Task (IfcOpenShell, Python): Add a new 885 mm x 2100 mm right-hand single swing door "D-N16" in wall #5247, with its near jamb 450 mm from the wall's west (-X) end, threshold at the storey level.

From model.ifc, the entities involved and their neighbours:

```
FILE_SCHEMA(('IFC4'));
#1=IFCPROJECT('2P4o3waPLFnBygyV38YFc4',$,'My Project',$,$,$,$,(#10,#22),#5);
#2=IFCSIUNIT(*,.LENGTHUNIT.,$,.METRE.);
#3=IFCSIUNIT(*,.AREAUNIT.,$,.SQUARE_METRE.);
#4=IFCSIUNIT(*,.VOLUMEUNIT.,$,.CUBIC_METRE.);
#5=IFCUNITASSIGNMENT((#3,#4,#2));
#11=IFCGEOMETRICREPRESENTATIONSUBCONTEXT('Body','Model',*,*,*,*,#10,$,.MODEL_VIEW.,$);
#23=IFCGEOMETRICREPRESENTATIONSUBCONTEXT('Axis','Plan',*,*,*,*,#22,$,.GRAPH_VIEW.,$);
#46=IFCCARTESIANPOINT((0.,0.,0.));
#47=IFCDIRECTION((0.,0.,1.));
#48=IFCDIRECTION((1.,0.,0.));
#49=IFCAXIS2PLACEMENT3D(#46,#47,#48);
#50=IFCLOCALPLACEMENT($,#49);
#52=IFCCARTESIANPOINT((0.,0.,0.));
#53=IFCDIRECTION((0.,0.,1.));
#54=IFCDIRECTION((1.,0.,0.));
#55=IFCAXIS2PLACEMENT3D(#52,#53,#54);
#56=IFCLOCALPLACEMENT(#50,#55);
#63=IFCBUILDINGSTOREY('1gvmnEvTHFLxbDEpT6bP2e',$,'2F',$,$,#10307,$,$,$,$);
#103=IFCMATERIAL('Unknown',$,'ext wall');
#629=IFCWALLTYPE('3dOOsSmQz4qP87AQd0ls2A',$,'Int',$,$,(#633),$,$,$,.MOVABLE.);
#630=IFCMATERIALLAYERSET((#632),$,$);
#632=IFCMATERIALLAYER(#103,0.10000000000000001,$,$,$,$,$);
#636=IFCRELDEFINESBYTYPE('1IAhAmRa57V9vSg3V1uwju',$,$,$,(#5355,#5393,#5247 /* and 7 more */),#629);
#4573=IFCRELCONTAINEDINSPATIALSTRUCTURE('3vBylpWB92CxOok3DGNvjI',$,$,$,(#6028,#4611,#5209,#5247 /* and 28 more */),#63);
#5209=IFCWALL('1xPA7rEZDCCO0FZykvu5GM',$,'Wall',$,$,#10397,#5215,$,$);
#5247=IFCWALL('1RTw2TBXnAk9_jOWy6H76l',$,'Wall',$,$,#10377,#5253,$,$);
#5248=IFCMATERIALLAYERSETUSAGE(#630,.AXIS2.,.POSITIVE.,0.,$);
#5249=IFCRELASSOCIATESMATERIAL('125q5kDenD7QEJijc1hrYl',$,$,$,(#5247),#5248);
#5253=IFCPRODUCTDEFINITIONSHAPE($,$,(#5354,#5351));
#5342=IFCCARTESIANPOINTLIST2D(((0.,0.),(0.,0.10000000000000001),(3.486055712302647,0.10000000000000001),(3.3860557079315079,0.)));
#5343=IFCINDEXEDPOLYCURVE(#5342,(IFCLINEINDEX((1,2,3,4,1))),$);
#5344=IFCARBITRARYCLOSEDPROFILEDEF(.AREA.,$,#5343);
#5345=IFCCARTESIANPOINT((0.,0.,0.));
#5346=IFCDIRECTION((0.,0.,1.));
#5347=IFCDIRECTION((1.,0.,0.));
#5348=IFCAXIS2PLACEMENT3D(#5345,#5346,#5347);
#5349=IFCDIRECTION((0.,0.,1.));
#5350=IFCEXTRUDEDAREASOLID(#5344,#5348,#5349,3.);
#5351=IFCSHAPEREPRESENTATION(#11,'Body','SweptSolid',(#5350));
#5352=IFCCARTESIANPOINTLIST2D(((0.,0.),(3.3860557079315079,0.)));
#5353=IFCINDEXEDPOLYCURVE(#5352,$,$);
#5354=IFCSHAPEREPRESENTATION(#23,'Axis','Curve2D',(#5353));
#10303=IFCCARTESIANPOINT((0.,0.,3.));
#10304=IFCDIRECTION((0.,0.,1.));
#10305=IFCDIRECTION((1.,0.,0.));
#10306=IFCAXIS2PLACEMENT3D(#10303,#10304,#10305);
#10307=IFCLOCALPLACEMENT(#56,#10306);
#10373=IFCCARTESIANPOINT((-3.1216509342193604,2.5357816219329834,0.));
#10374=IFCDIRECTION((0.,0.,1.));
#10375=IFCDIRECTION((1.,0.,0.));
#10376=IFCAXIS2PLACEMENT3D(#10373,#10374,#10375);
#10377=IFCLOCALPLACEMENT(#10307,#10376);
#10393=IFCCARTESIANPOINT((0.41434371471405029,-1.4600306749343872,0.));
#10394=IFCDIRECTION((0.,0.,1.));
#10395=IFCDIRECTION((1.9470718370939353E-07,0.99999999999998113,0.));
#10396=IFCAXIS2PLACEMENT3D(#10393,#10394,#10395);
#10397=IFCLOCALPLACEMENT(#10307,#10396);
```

```python
import numpy as np
import ifcopenshell
import ifcopenshell.api.feature
import ifcopenshell.api.geometry
import ifcopenshell.api.root
import ifcopenshell.api.spatial
import ifcopenshell.geom
import ifcopenshell.util.element
import ifcopenshell.util.placement
import ifcopenshell.util.representation
import ifcopenshell.util.shape
import ifcopenshell.util.unit

model = ifcopenshell.open("model.ifc")
unit_scale = ifcopenshell.util.unit.calculate_unit_scale(model)
settings = ifcopenshell.geom.settings()


def volume(element):
    """Net volume in cubic metres, openings subtracted."""
    shape = ifcopenshell.geom.create_shape(settings, element)
    return ifcopenshell.util.shape.get_volume(shape.geometry)


wall = model.by_guid("1RTw2TBXnAk9_jOWy6H76l")
storey = ifcopenshell.util.element.get_container(wall, ifc_class="IfcBuildingStorey")
context = ifcopenshell.util.representation.get_context(model, "Model", "Body", "MODEL_VIEW")
before = volume(wall)

width, height, from_end, sill = 0.885, 2.1, 0.45, 0.0  # metres

# The wall runs along its own X axis, and the end named is its -X end.
wall_shape = ifcopenshell.geom.create_shape(settings, wall)
x, y, z = ifcopenshell.util.shape.get_vertices(wall_shape.geometry).T
start = x.min() + from_end
face, thickness = float(y.min()), float(y.max() - y.min())
wall_matrix = ifcopenshell.util.placement.get_local_placement(wall.ObjectPlacement)
level = ifcopenshell.util.placement.get_local_placement(storey.ObjectPlacement)[2, 3]


def in_wall(x, y):
    """Placement at x, y metres in the wall's axes, at sill height."""
    matrix = wall_matrix.copy()
    matrix[:, 3] = wall_matrix @ np.array([x / unit_scale, y / unit_scale, 0.0, 1.0])
    matrix[2, 3] = level + sill / unit_scale
    return matrix


# Opening: a box that overshoots both wall faces by 50 mm.
opening = ifcopenshell.api.root.create_entity(model, ifc_class="IfcOpeningElement", predefined_type="OPENING")
box = ifcopenshell.api.geometry.add_wall_representation(
    model, context=context, length=width, height=height, thickness=thickness + 0.1
)
ifcopenshell.api.geometry.assign_representation(model, product=opening, representation=box)
ifcopenshell.api.geometry.edit_object_placement(model, product=opening, matrix=in_wall(start, face - 0.05), is_si=False)
ifcopenshell.api.feature.add_feature(model, feature=opening, element=wall)

door = ifcopenshell.api.root.create_entity(model, ifc_class="IfcDoor", name="D-N16", predefined_type="DOOR")
door.OverallWidth, door.OverallHeight = width / unit_scale, height / unit_scale
door.OperationType = "SINGLE_SWING_RIGHT"
body = ifcopenshell.api.geometry.add_door_representation(
    model,
    context=context,
    overall_width=door.OverallWidth,
    overall_height=door.OverallHeight,
    operation_type="SINGLE_SWING_RIGHT",
    lining_properties={"LiningDepth": thickness / unit_scale, "ThresholdDepth": thickness / unit_scale},
)
ifcopenshell.api.geometry.assign_representation(model, product=door, representation=body)
ifcopenshell.api.spatial.assign_container(model, products=[door], relating_structure=storey)
ifcopenshell.api.feature.add_filling(model, opening=opening, element=door)

# The lining spans the wall, so the door starts at the wall face.
ifcopenshell.api.geometry.edit_object_placement(model, product=door, matrix=in_wall(start, face), is_si=False)

after = volume(wall)

print(f"wall volume {before:.3f} -> {after:.3f} m3")

model.write("model_rev.ifc")
```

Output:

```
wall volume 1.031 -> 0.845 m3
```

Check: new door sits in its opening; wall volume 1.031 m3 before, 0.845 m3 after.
